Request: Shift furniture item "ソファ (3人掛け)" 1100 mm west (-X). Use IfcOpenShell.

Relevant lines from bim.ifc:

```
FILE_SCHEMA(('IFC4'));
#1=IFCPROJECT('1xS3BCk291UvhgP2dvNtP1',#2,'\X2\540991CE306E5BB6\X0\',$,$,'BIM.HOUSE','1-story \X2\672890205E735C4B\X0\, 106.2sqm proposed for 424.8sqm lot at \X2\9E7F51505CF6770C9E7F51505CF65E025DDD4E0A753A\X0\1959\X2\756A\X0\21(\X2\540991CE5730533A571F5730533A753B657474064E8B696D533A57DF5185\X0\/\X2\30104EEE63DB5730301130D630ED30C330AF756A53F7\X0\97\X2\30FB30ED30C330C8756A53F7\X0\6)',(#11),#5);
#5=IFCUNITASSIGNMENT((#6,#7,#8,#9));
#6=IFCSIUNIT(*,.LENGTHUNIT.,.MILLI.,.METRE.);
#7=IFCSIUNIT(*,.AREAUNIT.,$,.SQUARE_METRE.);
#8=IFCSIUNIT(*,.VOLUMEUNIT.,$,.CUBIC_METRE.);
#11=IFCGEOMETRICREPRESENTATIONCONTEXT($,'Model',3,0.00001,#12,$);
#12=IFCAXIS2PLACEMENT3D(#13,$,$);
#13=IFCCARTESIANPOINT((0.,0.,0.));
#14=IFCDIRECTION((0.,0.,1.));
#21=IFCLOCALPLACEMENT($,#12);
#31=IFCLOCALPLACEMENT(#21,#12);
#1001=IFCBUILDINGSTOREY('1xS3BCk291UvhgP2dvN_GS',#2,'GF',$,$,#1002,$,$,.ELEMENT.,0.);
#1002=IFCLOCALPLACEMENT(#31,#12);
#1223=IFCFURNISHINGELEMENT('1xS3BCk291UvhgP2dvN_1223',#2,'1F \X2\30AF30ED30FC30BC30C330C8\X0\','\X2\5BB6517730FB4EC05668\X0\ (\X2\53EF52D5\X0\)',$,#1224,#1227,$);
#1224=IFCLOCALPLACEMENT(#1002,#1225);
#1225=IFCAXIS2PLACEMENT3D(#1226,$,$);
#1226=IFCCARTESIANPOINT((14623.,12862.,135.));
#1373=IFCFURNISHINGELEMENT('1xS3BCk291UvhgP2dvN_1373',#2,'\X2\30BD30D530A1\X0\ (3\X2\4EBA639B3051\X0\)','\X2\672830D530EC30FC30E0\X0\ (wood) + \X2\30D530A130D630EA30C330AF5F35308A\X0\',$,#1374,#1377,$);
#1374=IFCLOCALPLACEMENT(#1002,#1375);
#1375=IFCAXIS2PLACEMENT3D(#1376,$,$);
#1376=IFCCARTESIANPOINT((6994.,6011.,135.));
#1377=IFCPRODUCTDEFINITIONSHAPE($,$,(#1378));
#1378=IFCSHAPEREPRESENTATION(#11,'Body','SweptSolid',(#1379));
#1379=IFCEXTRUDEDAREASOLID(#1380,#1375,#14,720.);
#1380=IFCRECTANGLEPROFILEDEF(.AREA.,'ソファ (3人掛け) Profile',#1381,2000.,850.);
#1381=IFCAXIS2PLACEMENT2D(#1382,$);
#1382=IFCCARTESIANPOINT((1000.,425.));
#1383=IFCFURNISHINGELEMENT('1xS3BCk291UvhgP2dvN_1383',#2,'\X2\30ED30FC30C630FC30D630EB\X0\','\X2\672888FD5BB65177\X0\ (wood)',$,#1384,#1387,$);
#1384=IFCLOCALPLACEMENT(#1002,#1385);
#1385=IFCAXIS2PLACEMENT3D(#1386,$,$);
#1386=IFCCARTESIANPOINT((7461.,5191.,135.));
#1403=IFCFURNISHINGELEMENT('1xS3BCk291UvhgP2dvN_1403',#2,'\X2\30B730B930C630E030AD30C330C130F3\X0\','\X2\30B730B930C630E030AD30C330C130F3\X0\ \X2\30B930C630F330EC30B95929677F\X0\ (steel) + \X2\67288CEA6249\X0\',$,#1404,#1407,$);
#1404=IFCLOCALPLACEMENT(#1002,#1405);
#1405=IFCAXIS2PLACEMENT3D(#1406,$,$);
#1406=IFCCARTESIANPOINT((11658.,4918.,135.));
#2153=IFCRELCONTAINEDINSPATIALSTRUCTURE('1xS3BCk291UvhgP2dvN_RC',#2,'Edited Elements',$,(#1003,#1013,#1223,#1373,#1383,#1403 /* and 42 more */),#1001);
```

```python
import ifcopenshell
import ifcopenshell.api.geometry
import ifcopenshell.util.placement
import ifcopenshell.util.unit

model = ifcopenshell.open("bim.ifc")
unit_scale = ifcopenshell.util.unit.calculate_unit_scale(model)

item = model.by_guid("1xS3BCk291UvhgP2dvN_1373")
matrix = ifcopenshell.util.placement.get_local_placement(item.ObjectPlacement)
matrix[0, 3] -= 1.1 / unit_scale
ifcopenshell.api.geometry.edit_object_placement(model, product=item, matrix=matrix, is_si=False)

print(ifcopenshell.util.placement.get_local_placement(item.ObjectPlacement).round(3) + 0.0)

model.write("bim_rev.ifc")
```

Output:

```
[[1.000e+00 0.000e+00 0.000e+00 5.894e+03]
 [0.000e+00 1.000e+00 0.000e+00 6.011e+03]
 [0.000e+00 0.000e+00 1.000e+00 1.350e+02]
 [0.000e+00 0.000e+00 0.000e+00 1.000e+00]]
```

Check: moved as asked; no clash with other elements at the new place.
